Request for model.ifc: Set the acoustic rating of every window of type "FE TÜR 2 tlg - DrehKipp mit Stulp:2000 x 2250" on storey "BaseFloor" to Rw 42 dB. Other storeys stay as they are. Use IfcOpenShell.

First a look at what the model holds.

```python
import ifcopenshell
import ifcopenshell.util.element

model = ifcopenshell.open("model.ifc")
print(model.schema)
storey = next(s for s in model.by_type("IfcBuildingStorey") if s.Name == "BaseFloor")
windows = [e for e in ifcopenshell.util.element.get_decomposition(storey) if e.is_a("IfcWindow")]
seen = {}
for e in windows:
    element_type = ifcopenshell.util.element.get_type(e)
    key = (element_type.Name if element_type != e and element_type else None, ifcopenshell.util.element.get_pset(e, "Pset_WindowCommon", "AcousticRating"))
    seen[key] = seen.get(key, 0) + 1
for (name, value), count in sorted(seen.items(), key=str):
    print(count, "x", name, "|", value)
```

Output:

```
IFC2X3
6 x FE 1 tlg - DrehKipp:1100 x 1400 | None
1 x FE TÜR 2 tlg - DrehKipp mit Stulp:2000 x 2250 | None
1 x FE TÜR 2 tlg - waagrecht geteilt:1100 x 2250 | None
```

```python
import ifcopenshell
import ifcopenshell.api.pset
import ifcopenshell.util.element

model = ifcopenshell.open("model.ifc")

storey = next(s for s in model.by_type("IfcBuildingStorey") if s.Name == "BaseFloor")
windows = [e for e in ifcopenshell.util.element.get_decomposition(storey) if e.is_a("IfcWindow")]

count = 0
for e in windows:
    element_type = ifcopenshell.util.element.get_type(e)
    if element_type in (None, e) or element_type.Name != "FE TÜR 2 tlg - DrehKipp mit Stulp:2000 x 2250":
        continue
    # add_pset returns the element's existing set when there is one.
    pset = ifcopenshell.api.pset.add_pset(model, product=e, name="Pset_WindowCommon")
    ifcopenshell.api.pset.edit_pset(model, pset=pset, properties={"AcousticRating": "Rw 42 dB"})
    count += 1

print(count, "windows updated")

model.write("model-out.ifc")
```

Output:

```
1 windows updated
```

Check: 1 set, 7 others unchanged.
